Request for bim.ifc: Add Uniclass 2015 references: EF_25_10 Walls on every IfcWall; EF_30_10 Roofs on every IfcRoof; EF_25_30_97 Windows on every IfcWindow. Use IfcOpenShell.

First a look at what the model holds.

```python
import ifcopenshell

model = ifcopenshell.open("bim.ifc")
print(model.schema)
print("classifications:", [c.Name for c in model.by_type("IfcClassification")])
for ifc_class in ("IfcDoor", "IfcRoof", "IfcStair", "IfcWall", "IfcWindow"):
    print(ifc_class, len(model.by_type(ifc_class)))
```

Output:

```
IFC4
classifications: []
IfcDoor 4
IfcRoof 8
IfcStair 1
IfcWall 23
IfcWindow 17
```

```python
import ifcopenshell
import ifcopenshell.api.classification

model = ifcopenshell.open("bim.ifc")

system = ifcopenshell.api.classification.add_classification(model, classification="Uniclass 2015")

codes = {
    "IfcWall": ("EF_25_10", "Walls"),
    "IfcRoof": ("EF_30_10", "Roofs"),
    "IfcWindow": ("EF_25_30_97", "Windows"),
}
for ifc_class, (code, name) in codes.items():
    products = model.by_type(ifc_class)
    ifcopenshell.api.classification.add_reference(
        model, products=products, classification=system, identification=code, name=name
    )
    print(code, len(products))

model.write("bim_rev.ifc")
```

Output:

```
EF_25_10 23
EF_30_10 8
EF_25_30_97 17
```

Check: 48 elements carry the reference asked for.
